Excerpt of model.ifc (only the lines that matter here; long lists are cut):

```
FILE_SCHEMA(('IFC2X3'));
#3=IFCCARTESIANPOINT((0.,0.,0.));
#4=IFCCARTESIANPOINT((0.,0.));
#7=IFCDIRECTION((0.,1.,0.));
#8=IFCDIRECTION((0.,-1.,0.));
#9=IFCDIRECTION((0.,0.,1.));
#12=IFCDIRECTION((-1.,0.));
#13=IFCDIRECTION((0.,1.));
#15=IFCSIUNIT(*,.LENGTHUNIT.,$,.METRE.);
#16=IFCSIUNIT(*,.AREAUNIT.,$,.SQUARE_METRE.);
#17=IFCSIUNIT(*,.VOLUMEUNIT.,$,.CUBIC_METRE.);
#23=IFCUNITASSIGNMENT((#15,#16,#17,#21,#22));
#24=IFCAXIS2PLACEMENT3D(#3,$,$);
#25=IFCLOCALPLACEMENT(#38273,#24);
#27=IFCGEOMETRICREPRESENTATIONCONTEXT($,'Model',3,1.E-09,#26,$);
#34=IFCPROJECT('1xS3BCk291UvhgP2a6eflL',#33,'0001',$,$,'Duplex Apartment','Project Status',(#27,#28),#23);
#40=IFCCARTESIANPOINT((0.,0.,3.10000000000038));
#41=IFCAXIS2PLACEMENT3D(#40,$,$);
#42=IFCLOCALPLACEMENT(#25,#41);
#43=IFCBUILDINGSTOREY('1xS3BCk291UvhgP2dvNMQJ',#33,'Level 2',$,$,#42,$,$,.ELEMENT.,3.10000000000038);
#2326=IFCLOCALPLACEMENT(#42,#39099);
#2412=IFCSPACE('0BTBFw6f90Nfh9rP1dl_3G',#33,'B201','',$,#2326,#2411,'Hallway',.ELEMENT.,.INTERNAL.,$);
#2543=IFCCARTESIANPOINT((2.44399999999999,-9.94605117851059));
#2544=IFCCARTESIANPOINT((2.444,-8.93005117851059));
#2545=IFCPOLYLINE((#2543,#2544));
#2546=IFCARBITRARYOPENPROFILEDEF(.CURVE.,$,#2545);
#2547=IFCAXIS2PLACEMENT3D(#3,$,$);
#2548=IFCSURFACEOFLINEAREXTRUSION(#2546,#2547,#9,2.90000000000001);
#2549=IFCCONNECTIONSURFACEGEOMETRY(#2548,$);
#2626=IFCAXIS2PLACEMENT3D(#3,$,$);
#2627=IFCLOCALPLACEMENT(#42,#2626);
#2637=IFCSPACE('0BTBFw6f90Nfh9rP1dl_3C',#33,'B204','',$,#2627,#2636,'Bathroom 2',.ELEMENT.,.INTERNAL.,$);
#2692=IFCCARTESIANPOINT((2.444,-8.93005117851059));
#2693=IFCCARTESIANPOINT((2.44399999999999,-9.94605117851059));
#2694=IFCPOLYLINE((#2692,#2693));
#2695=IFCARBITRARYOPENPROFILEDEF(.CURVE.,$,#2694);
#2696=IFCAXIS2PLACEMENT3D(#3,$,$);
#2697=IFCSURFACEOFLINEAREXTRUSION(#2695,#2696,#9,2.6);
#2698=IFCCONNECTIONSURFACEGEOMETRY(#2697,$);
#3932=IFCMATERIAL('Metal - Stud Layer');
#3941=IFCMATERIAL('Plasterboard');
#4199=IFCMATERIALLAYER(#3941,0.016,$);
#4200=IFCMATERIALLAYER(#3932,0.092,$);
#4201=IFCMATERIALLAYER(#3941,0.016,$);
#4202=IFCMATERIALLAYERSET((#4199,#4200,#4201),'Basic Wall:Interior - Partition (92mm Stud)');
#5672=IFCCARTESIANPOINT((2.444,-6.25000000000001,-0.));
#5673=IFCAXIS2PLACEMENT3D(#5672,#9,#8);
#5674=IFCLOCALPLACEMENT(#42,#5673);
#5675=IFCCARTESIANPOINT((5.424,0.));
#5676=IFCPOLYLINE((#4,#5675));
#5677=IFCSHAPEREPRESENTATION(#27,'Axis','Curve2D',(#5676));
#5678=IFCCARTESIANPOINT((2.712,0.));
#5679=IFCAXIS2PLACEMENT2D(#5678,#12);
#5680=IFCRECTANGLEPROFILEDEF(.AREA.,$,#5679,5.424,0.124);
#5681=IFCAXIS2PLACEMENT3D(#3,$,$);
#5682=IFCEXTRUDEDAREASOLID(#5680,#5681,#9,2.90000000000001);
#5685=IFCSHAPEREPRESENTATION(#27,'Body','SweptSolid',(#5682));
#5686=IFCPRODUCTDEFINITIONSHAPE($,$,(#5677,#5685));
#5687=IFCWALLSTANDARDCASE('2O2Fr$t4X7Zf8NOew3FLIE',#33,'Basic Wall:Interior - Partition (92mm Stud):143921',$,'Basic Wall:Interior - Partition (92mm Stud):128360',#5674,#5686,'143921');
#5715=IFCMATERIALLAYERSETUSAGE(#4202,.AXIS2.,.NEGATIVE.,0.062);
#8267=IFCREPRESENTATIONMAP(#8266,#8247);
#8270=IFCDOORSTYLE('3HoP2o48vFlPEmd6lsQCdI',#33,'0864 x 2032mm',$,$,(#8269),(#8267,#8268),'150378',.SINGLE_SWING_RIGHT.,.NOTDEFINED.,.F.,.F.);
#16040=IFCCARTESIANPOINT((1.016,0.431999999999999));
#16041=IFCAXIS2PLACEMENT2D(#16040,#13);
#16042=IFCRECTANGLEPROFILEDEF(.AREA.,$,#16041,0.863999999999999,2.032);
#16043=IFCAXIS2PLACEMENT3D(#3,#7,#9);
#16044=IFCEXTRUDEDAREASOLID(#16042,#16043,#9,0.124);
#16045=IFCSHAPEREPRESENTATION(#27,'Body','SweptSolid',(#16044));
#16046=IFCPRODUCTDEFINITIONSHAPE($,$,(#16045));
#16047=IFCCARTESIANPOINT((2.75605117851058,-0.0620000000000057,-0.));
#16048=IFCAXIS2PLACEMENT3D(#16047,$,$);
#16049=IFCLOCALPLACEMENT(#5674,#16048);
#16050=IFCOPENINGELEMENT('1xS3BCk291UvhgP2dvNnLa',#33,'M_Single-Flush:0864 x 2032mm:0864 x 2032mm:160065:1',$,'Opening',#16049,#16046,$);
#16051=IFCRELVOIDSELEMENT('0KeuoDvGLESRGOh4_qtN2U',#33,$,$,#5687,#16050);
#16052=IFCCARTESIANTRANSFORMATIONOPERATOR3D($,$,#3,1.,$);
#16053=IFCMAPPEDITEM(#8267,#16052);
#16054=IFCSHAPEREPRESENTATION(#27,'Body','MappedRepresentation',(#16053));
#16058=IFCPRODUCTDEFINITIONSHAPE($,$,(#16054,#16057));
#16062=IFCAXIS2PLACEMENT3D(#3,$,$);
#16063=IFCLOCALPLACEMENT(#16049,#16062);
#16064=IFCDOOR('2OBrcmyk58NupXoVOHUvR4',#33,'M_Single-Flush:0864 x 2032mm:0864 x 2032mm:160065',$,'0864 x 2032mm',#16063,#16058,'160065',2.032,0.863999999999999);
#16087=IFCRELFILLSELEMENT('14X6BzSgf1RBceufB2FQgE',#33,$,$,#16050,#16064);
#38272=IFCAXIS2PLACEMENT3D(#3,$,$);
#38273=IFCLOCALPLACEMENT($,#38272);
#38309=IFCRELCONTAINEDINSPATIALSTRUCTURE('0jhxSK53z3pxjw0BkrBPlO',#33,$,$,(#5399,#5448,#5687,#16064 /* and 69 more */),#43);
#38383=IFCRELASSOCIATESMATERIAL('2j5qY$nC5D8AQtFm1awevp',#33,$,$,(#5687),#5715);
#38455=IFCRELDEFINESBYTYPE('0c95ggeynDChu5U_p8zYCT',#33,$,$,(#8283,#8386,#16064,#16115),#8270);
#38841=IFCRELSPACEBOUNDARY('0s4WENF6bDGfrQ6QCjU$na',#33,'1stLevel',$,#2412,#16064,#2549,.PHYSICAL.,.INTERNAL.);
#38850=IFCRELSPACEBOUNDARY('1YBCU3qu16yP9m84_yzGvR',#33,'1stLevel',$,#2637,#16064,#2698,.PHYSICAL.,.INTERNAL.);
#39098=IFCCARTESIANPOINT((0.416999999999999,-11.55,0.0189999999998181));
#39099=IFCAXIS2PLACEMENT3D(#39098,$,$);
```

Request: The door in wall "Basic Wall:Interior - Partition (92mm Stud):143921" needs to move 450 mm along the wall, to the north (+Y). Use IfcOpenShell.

```python
import numpy as np
import ifcopenshell
import ifcopenshell.api.geometry
import ifcopenshell.util.placement

model = ifcopenshell.open("model.ifc")

door = model.by_id(16064)
opening = door.FillsVoids[0].RelatingOpeningElement
wall = opening.VoidsElements[0].RelatingBuildingElement

wall_matrix = ifcopenshell.util.placement.get_local_placement(wall.ObjectPlacement)
shift = wall_matrix[:3, 0] * -0.45
before = ifcopenshell.util.placement.get_local_placement(door.ObjectPlacement)[:3, 3].copy()

# The door is placed relative to its opening, so it follows when the opening moves.
matrix = ifcopenshell.util.placement.get_local_placement(opening.ObjectPlacement)
matrix[:3, 3] += shift
ifcopenshell.api.geometry.edit_object_placement(
    model, product=opening, matrix=matrix, is_si=False, should_transform_children=True
)

# Space boundary surfaces are stored in each space's coordinates; move them too.
for rel in door.ProvidesBoundaries:
    if not rel.ConnectionGeometry:
        continue
    surface = rel.ConnectionGeometry.SurfaceOnRelatingElement
    space_matrix = ifcopenshell.util.placement.get_local_placement(rel.RelatingSpace.ObjectPlacement)
    point = np.array(surface.Position.Location.Coordinates) + space_matrix[:3, :3].T @ shift
    surface.Position = model.createIfcAxis2Placement3D(
        model.createIfcCartesianPoint(point.tolist()), surface.Position.Axis, surface.Position.RefDirection
    )

after = ifcopenshell.util.placement.get_local_placement(door.ObjectPlacement)[:3, 3]
print("door moved by", (after - before).round(3) + 0.0)

model.write("model-out.ifc")
```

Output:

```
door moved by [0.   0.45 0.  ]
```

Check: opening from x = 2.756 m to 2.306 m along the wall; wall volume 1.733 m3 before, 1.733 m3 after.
